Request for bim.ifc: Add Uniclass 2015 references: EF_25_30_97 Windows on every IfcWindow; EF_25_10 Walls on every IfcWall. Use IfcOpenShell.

First a look at what the model holds.

```python
import ifcopenshell

model = ifcopenshell.open("bim.ifc")
print(model.schema)
print("classifications:", [c.Name for c in model.by_type("IfcClassification")])
for ifc_class in ("IfcDoor", "IfcRoof", "IfcStair", "IfcWall", "IfcWindow"):
    print(ifc_class, len(model.by_type(ifc_class)))
```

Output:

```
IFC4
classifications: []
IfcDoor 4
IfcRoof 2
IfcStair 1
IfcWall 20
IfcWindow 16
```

```python
import ifcopenshell
import ifcopenshell.api.classification

model = ifcopenshell.open("bim.ifc")

system = ifcopenshell.api.classification.add_classification(model, classification="Uniclass 2015")

codes = {
    "IfcWindow": ("EF_25_30_97", "Windows"),
    "IfcWall": ("EF_25_10", "Walls"),
}
for ifc_class, (code, name) in codes.items():
    products = model.by_type(ifc_class)
    ifcopenshell.api.classification.add_reference(
        model, products=products, classification=system, identification=code, name=name
    )
    print(code, len(products))

model.write("bim_updated.ifc")
```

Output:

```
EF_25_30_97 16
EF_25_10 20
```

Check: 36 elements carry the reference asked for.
